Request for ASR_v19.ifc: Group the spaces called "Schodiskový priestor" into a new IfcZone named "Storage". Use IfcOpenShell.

First a look at what the model holds.

```python
import ifcopenshell

model = ifcopenshell.open("ASR_v19.ifc")
print(model.schema)
seen = {}
for space in model.by_type("IfcSpace"):
    seen[space.LongName] = seen.get(space.LongName, 0) + 1
for name, count in sorted(seen.items(), key=str):
    print(count, "x", name)
print("zones:", [z.Name for z in model.by_type("IfcZone")][:20])
```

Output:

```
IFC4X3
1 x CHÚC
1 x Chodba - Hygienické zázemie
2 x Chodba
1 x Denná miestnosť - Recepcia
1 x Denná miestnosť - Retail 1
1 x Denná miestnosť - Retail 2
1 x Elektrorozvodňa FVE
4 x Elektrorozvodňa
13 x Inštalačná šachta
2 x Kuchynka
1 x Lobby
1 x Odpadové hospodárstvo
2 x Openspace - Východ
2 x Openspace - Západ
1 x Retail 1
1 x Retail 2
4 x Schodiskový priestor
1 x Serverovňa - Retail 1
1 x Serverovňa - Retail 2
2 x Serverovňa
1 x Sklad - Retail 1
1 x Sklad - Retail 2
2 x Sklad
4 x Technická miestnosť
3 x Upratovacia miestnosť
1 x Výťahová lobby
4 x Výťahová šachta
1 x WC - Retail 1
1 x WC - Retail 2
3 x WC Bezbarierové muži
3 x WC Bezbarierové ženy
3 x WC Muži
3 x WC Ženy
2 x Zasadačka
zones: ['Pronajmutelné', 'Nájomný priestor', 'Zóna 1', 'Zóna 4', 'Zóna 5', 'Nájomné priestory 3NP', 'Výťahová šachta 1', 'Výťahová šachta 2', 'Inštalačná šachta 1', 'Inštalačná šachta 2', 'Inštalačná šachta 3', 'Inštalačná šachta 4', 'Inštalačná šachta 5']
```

```python
import ifcopenshell
import ifcopenshell.api.group
import ifcopenshell.api.root

model = ifcopenshell.open("ASR_v19.ifc")

names = {"Schodiskový priestor"}
spaces = [s for s in model.by_type("IfcSpace") if s.LongName in names]

zone = ifcopenshell.api.root.create_entity(model, ifc_class="IfcZone", name="Storage")
ifcopenshell.api.group.assign_group(model, products=spaces, group=zone)
print(len(spaces), "spaces in", zone.Name)

model.write("ASR_v19_rev.ifc")
```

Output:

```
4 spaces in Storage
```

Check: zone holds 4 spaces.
